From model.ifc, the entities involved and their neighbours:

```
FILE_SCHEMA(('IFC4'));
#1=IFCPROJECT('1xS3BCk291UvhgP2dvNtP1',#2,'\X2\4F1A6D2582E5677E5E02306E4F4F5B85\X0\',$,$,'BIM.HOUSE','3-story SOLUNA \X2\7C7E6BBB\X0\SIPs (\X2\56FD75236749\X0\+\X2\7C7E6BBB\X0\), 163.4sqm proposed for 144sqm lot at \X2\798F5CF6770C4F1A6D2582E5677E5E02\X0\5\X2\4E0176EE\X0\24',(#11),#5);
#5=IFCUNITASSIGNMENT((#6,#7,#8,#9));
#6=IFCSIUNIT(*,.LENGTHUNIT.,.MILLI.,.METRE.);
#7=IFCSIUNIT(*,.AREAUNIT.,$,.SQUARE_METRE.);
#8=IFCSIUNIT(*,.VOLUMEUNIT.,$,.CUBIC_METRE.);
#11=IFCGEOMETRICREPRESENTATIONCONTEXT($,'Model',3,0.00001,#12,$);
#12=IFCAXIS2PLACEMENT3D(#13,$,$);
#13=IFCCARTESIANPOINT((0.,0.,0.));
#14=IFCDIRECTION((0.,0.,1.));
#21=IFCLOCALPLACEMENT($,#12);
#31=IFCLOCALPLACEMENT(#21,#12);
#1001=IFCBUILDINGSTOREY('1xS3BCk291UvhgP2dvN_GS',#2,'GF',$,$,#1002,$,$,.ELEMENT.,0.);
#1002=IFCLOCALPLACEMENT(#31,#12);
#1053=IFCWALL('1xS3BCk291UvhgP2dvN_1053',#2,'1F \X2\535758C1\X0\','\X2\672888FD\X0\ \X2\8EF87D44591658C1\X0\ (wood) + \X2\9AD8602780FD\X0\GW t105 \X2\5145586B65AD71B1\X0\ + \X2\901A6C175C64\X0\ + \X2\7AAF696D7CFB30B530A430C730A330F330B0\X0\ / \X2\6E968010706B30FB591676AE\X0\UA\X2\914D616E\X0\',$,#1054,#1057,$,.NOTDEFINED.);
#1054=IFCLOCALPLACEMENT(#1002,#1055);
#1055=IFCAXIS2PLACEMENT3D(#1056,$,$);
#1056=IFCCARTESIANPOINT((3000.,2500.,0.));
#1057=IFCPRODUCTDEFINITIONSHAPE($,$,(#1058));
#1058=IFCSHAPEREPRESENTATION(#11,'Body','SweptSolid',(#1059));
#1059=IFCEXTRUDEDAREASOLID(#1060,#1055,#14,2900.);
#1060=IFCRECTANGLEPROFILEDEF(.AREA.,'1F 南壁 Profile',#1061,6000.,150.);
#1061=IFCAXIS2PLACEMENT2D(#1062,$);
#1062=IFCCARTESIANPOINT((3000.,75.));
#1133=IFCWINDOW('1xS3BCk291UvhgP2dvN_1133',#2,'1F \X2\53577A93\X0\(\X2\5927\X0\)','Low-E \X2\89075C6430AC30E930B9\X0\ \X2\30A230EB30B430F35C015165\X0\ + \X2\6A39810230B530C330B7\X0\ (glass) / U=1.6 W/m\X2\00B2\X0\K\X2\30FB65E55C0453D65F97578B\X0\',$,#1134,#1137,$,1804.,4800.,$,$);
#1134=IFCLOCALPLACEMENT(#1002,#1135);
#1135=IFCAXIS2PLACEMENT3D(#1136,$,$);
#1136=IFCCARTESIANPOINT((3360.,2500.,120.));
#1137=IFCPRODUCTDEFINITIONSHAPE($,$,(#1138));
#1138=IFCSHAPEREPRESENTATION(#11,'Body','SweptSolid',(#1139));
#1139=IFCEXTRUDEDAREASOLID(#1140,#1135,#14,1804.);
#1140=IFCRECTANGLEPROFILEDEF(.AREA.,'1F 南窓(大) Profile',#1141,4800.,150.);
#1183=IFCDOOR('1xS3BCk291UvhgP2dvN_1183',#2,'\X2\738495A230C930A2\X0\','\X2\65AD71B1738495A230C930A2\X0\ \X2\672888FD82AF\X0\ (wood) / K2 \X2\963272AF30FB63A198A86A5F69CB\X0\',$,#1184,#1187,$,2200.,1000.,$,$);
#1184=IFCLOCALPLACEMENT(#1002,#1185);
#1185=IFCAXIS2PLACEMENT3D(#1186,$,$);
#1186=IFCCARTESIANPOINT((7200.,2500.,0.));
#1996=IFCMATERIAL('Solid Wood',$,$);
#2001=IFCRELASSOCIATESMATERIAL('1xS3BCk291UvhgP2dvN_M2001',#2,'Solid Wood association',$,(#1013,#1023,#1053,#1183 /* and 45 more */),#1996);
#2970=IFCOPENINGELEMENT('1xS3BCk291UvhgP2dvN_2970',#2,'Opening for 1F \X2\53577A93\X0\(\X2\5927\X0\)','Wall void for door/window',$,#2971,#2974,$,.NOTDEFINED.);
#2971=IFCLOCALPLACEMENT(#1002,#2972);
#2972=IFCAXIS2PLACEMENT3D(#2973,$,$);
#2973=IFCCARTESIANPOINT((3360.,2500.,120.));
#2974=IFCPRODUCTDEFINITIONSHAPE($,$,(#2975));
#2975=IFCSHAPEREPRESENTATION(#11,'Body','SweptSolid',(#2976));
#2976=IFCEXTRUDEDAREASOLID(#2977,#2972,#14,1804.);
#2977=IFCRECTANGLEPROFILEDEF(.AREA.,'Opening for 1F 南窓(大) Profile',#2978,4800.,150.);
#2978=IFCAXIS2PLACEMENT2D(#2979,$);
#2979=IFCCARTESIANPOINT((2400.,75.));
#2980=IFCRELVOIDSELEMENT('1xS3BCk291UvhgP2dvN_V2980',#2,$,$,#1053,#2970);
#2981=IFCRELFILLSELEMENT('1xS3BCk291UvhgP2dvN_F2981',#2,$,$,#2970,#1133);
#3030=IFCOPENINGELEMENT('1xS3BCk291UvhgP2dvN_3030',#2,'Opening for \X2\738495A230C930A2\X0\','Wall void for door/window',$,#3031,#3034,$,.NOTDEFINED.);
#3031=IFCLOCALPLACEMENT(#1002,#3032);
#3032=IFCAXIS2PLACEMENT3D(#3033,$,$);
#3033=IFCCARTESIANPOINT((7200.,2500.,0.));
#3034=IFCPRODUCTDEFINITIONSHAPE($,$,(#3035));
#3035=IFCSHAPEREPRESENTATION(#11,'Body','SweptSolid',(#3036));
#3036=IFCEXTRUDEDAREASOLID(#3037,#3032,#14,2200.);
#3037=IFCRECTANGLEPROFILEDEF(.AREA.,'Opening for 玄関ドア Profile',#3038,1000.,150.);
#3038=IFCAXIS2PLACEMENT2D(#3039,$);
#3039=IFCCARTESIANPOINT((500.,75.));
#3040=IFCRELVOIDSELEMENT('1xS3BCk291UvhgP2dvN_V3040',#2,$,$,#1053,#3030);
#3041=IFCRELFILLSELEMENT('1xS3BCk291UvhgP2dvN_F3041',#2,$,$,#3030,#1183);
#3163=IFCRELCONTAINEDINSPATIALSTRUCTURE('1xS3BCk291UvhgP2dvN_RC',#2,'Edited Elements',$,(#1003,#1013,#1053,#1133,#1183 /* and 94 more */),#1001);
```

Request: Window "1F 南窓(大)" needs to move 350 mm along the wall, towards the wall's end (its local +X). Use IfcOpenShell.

```python
import ifcopenshell
import ifcopenshell.api.geometry
import ifcopenshell.util.placement
import ifcopenshell.util.unit

model = ifcopenshell.open("model.ifc")
unit_scale = ifcopenshell.util.unit.calculate_unit_scale(model)

window = model.by_id(1133)
opening = window.FillsVoids[0].RelatingOpeningElement
wall = opening.VoidsElements[0].RelatingBuildingElement

wall_matrix = ifcopenshell.util.placement.get_local_placement(wall.ObjectPlacement)
shift = wall_matrix[:3, 0] * 0.35 / unit_scale
before = ifcopenshell.util.placement.get_local_placement(window.ObjectPlacement)[:3, 3].copy()

# The window is not placed relative to its opening, so move both.
for product in (opening, window):
    matrix = ifcopenshell.util.placement.get_local_placement(product.ObjectPlacement)
    matrix[:3, 3] += shift
    ifcopenshell.api.geometry.edit_object_placement(model, product=product, matrix=matrix, is_si=False)

after = ifcopenshell.util.placement.get_local_placement(window.ObjectPlacement)[:3, 3]
print("window moved by", (after - before).round(3) + 0.0)

model.write("model_v2.ifc")
```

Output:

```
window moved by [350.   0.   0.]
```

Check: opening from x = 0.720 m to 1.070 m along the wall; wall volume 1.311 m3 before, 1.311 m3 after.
